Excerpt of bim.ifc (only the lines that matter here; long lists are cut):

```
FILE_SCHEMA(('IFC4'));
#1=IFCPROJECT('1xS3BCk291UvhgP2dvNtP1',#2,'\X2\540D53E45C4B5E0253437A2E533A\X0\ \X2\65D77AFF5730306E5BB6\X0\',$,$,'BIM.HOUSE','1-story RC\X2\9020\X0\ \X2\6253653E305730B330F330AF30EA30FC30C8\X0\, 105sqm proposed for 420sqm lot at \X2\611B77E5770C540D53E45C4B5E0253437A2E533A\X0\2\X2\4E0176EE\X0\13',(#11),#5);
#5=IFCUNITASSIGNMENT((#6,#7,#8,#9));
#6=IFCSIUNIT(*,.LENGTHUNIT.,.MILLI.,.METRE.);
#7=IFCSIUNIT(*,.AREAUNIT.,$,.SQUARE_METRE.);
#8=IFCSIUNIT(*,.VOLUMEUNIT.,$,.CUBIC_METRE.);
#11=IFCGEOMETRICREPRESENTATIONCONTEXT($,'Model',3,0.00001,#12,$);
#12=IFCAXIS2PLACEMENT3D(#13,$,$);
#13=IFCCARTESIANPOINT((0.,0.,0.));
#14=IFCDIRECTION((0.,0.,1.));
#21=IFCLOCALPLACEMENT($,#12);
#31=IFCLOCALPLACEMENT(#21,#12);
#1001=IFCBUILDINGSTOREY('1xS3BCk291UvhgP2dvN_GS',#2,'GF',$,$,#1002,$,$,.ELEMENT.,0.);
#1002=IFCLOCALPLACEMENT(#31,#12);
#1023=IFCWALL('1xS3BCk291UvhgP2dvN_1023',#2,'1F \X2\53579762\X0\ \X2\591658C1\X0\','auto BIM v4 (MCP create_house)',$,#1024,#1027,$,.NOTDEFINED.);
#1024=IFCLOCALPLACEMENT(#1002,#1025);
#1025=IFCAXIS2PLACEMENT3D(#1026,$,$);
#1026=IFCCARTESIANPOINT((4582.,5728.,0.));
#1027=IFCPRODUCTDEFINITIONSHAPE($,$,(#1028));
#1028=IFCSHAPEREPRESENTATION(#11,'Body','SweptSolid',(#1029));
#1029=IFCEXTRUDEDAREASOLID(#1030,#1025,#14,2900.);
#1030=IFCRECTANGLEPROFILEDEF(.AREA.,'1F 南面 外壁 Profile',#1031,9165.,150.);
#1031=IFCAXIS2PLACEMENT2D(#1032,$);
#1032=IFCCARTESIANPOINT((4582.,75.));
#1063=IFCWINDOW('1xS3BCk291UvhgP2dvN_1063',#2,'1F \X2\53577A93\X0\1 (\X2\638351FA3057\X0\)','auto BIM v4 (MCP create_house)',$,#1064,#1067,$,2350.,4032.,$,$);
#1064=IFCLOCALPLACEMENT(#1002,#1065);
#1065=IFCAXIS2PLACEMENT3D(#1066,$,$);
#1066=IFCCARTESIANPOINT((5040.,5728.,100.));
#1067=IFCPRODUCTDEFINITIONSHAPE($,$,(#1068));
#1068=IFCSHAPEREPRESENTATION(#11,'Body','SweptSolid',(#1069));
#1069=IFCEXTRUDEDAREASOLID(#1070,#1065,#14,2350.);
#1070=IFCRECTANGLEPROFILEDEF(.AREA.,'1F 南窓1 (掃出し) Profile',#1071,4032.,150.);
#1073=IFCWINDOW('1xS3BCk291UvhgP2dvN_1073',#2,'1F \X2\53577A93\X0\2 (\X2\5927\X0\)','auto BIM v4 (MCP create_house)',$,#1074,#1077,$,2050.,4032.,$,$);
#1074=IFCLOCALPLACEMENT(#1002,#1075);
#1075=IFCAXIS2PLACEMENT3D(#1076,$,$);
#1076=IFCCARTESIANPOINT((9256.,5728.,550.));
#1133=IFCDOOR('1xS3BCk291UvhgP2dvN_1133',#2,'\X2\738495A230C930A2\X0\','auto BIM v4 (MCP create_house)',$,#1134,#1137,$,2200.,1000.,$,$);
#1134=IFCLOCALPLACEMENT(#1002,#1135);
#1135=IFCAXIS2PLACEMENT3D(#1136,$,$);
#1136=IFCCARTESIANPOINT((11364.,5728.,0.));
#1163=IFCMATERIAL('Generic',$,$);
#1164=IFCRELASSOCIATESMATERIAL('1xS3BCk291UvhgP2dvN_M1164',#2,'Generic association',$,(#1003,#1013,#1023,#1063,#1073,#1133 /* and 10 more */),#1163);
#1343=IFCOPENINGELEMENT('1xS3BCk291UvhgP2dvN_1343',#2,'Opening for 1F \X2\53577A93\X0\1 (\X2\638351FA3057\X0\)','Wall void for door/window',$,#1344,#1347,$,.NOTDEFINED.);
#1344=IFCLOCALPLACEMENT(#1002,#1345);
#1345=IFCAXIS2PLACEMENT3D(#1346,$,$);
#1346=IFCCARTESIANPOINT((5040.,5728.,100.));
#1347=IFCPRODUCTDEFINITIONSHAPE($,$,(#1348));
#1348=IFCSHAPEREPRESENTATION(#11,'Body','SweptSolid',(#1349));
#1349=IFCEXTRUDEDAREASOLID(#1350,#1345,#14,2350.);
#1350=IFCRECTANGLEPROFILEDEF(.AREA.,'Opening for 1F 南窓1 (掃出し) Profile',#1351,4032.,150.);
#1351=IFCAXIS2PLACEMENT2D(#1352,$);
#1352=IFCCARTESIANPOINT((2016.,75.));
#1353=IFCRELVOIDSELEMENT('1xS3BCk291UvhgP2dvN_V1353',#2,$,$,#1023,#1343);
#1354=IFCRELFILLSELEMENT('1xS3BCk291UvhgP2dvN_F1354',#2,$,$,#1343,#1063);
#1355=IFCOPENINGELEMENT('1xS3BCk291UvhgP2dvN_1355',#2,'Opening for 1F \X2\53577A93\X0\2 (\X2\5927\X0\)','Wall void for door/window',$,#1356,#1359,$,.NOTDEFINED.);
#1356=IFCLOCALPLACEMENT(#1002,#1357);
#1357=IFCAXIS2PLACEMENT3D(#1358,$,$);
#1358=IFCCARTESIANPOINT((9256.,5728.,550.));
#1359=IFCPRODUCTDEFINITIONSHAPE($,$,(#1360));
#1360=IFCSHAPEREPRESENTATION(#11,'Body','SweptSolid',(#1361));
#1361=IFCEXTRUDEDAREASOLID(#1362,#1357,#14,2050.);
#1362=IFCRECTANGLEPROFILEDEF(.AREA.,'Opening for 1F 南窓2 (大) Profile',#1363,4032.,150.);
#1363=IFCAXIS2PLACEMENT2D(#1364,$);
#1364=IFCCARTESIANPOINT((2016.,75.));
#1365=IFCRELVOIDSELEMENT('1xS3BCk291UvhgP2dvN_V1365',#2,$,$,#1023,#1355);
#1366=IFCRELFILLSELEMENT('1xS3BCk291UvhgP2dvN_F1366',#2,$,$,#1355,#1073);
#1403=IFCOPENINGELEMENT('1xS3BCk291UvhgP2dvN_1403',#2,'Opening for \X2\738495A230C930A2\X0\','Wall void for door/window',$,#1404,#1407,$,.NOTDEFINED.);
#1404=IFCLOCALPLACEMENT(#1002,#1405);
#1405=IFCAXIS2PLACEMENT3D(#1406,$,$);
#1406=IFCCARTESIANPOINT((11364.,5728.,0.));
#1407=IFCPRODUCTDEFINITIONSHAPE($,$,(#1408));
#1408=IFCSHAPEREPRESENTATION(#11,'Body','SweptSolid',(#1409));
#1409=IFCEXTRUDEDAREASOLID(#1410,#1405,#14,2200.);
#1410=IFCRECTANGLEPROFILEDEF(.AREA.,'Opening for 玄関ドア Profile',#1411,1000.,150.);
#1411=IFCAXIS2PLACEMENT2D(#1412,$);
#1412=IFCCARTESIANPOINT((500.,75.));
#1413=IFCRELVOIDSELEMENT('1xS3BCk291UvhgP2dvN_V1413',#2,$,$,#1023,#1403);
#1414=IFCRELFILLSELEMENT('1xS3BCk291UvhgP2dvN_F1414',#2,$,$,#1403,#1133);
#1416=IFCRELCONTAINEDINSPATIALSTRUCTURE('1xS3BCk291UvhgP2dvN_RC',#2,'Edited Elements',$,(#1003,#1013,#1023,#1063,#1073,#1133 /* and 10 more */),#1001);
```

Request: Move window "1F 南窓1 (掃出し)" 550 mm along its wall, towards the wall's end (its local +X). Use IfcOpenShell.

```python
import ifcopenshell
import ifcopenshell.api.geometry
import ifcopenshell.util.placement

model = ifcopenshell.open("bim.ifc")

window = model.by_guid("1xS3BCk291UvhgP2dvN_1063")
opening = window.FillsVoids[0].RelatingOpeningElement
wall = opening.VoidsElements[0].RelatingBuildingElement

wall_matrix = ifcopenshell.util.placement.get_local_placement(wall.ObjectPlacement)
shift = wall_matrix[:3, 0] * 550.0
before = ifcopenshell.util.placement.get_local_placement(window.ObjectPlacement)[:3, 3].copy()

# The window is not placed relative to its opening, so move both.
for product in (opening, window):
    matrix = ifcopenshell.util.placement.get_local_placement(product.ObjectPlacement)
    matrix[:3, 3] += shift
    ifcopenshell.api.geometry.edit_object_placement(model, product=product, matrix=matrix, is_si=False)

after = ifcopenshell.util.placement.get_local_placement(window.ObjectPlacement)[:3, 3]
print("window moved by", (after - before).round(3) + 0.0)

model.write("bim_updated.ifc")
```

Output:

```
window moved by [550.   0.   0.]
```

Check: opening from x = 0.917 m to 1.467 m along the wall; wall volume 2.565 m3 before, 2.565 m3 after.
